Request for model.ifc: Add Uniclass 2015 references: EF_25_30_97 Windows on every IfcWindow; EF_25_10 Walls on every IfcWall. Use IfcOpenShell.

First a look at what the model holds.

```python
import ifcopenshell

model = ifcopenshell.open("model.ifc")
print(model.schema)
print("classifications:", [c.Name for c in model.by_type("IfcClassification")])
for ifc_class in ("IfcDoor", "IfcRoof", "IfcStair", "IfcWall", "IfcWindow"):
    print(ifc_class, len(model.by_type(ifc_class)))
```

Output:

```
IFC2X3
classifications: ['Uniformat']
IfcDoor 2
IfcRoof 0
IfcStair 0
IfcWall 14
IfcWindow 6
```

```python
import ifcopenshell
import ifcopenshell.api.classification

model = ifcopenshell.open("model.ifc")

# IFC2X3 requires Source and Edition and has no link from the project to the system.
system = model.create_entity("IfcClassification", Source="NBS", Edition="2015", Name="Uniclass 2015")

codes = {
    "IfcWindow": ("EF_25_30_97", "Windows"),
    "IfcWall": ("EF_25_10", "Walls"),
}
for ifc_class, (code, name) in codes.items():
    products = model.by_type(ifc_class)
    ifcopenshell.api.classification.add_reference(
        model, products=products, classification=system, identification=code, name=name
    )
    print(code, len(products))

model.write("model_v2.ifc")
```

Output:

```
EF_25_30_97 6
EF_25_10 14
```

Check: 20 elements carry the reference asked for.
